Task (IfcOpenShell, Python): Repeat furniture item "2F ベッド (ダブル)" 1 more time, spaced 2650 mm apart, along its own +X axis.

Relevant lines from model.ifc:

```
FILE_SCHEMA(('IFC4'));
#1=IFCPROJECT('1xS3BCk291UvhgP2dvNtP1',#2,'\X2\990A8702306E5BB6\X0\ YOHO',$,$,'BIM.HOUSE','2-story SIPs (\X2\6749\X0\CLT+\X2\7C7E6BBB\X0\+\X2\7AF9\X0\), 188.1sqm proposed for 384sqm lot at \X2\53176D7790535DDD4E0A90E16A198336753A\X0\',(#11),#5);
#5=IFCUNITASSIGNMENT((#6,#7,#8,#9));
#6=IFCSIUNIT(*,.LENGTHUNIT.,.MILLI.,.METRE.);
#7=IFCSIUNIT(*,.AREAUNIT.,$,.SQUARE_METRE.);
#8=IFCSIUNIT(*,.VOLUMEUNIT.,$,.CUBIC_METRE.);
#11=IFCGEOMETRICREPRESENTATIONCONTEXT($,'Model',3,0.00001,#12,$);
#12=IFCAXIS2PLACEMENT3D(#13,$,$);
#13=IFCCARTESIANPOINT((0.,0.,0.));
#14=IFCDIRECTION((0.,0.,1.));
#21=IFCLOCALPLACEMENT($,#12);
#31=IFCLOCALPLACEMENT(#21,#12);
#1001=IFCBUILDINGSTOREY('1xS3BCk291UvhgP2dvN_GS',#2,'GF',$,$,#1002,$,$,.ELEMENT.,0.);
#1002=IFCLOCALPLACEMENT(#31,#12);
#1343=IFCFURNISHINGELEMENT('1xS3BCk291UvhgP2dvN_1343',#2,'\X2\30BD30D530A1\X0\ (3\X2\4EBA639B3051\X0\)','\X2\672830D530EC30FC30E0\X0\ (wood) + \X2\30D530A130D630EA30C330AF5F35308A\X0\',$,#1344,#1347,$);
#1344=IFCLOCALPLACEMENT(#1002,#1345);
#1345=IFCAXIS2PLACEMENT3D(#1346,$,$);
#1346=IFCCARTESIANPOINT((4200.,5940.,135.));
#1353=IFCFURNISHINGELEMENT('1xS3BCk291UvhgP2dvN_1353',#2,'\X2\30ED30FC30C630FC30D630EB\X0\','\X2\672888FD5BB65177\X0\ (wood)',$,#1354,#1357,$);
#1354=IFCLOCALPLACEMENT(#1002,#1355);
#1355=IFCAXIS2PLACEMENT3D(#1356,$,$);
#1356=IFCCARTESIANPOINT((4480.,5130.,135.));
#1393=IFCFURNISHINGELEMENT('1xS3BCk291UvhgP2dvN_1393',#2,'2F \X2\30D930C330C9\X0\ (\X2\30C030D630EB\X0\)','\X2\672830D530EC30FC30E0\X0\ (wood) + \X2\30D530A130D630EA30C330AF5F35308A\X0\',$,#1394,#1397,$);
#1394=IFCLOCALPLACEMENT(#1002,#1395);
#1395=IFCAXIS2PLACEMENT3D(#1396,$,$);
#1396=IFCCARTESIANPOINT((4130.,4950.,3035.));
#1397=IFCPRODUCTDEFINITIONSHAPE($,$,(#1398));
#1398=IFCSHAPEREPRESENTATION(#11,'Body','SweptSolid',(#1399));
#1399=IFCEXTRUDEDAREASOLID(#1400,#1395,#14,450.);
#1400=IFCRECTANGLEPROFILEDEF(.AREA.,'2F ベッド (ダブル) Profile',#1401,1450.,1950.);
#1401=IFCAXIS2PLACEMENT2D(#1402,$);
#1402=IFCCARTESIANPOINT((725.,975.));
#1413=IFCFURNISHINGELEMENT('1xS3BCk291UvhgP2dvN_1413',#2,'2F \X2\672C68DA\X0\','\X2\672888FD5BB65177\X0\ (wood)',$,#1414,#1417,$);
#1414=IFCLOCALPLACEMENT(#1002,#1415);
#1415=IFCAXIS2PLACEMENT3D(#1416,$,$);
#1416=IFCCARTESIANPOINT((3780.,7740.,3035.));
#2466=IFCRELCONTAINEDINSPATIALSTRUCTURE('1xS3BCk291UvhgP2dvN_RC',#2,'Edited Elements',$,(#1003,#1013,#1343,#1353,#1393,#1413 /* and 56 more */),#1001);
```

```python
import ifcopenshell
import ifcopenshell.api.geometry
import ifcopenshell.api.root
import ifcopenshell.util.element
import ifcopenshell.util.placement

model = ifcopenshell.open("model.ifc")


def reuse_history(source, copy):
    """copy_class also copies each property set's owner history, people and application; keep the originals."""
    for rel in copy.IsDefinedBy:
        if rel.is_a("IfcRelDefinesByProperties") and (history := rel.RelatingPropertyDefinition.OwnerHistory):
            rel.RelatingPropertyDefinition.OwnerHistory = source.OwnerHistory
            ifcopenshell.util.element.remove_deep2(model, history)


source = model.by_guid("1xS3BCk291UvhgP2dvN_1393")
base = ifcopenshell.util.placement.get_local_placement(source.ObjectPlacement)
step = base[:3, 0] * 2650.0

for i in range(1, 2):
    copy = ifcopenshell.api.root.copy_class(model, product=source)
    copy.Representation = ifcopenshell.util.element.copy_deep(
        model, source.Representation, exclude=["IfcGeometricRepresentationContext", "IfcRepresentationMap"]
    )
    reuse_history(source, copy)
    matrix = base.copy()
    matrix[:3, 3] += i * step
    print("added at", matrix[:3, 3].round(3) + 0.0)
    ifcopenshell.api.geometry.edit_object_placement(model, product=copy, matrix=matrix, is_si=False)

model.write("model_edited.ifc")
```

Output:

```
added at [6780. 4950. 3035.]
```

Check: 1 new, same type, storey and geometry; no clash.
